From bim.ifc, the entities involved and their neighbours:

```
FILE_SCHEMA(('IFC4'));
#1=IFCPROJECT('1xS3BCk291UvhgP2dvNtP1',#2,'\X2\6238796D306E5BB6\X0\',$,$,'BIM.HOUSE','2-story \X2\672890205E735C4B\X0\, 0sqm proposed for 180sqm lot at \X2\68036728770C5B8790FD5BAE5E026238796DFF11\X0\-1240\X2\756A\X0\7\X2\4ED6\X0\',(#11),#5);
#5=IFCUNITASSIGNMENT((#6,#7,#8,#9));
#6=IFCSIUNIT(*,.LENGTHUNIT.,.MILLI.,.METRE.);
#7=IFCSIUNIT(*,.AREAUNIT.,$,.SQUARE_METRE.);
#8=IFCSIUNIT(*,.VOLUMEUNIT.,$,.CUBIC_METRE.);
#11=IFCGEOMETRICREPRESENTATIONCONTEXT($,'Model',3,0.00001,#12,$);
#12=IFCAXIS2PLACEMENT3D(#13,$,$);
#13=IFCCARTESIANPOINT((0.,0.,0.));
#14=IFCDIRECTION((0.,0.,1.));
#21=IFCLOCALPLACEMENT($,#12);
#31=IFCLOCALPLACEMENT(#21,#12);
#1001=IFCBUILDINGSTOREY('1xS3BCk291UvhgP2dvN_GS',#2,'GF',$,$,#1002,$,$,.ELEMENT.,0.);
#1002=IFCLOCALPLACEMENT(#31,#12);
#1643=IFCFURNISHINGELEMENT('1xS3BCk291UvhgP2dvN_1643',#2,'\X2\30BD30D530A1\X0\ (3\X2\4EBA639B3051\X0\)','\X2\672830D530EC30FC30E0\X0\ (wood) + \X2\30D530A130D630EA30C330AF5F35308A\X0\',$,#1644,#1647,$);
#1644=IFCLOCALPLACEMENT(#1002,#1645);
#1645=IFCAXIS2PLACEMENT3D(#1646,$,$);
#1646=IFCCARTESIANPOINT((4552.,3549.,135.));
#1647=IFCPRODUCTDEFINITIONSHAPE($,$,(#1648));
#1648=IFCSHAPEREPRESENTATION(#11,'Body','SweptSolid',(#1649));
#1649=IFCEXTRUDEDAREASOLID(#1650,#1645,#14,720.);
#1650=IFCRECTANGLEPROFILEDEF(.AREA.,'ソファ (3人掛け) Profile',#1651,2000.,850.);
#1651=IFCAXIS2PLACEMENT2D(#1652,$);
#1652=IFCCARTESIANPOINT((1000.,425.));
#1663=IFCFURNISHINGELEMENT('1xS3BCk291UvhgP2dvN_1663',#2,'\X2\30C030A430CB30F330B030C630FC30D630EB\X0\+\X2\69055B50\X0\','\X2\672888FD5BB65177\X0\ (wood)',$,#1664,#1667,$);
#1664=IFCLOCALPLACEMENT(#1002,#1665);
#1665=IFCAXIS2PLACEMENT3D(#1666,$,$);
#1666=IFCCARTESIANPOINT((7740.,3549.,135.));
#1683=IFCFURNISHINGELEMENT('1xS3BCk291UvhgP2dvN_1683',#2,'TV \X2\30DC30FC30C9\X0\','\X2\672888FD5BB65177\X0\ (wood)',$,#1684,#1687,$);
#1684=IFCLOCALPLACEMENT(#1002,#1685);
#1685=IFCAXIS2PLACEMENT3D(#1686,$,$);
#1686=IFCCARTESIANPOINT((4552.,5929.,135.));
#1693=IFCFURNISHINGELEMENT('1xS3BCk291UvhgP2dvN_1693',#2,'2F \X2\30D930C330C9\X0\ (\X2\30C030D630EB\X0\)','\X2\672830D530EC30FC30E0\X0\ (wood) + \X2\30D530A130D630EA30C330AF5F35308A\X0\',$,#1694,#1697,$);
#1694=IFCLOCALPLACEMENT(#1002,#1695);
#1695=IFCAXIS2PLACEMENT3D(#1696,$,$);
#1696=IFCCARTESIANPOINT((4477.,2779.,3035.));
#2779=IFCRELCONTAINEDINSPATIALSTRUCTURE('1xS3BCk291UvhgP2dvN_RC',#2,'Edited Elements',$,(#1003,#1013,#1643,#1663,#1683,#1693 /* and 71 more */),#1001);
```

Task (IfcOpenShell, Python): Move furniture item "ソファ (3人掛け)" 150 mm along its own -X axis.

```python
import ifcopenshell
import ifcopenshell.api.geometry
import ifcopenshell.util.placement
import ifcopenshell.util.unit

model = ifcopenshell.open("bim.ifc")
unit_scale = ifcopenshell.util.unit.calculate_unit_scale(model)

item = model.by_id(1643)
matrix = ifcopenshell.util.placement.get_local_placement(item.ObjectPlacement)
matrix[:3, 3] -= matrix[:3, 0] * 0.15 / unit_scale
ifcopenshell.api.geometry.edit_object_placement(model, product=item, matrix=matrix, is_si=False)

print(ifcopenshell.util.placement.get_local_placement(item.ObjectPlacement).round(3) + 0.0)

model.write("bim_v2.ifc")
```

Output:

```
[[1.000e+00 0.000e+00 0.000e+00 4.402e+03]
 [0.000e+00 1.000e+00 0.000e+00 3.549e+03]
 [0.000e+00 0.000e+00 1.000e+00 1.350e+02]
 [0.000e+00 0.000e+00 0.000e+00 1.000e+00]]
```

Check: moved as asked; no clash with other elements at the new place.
